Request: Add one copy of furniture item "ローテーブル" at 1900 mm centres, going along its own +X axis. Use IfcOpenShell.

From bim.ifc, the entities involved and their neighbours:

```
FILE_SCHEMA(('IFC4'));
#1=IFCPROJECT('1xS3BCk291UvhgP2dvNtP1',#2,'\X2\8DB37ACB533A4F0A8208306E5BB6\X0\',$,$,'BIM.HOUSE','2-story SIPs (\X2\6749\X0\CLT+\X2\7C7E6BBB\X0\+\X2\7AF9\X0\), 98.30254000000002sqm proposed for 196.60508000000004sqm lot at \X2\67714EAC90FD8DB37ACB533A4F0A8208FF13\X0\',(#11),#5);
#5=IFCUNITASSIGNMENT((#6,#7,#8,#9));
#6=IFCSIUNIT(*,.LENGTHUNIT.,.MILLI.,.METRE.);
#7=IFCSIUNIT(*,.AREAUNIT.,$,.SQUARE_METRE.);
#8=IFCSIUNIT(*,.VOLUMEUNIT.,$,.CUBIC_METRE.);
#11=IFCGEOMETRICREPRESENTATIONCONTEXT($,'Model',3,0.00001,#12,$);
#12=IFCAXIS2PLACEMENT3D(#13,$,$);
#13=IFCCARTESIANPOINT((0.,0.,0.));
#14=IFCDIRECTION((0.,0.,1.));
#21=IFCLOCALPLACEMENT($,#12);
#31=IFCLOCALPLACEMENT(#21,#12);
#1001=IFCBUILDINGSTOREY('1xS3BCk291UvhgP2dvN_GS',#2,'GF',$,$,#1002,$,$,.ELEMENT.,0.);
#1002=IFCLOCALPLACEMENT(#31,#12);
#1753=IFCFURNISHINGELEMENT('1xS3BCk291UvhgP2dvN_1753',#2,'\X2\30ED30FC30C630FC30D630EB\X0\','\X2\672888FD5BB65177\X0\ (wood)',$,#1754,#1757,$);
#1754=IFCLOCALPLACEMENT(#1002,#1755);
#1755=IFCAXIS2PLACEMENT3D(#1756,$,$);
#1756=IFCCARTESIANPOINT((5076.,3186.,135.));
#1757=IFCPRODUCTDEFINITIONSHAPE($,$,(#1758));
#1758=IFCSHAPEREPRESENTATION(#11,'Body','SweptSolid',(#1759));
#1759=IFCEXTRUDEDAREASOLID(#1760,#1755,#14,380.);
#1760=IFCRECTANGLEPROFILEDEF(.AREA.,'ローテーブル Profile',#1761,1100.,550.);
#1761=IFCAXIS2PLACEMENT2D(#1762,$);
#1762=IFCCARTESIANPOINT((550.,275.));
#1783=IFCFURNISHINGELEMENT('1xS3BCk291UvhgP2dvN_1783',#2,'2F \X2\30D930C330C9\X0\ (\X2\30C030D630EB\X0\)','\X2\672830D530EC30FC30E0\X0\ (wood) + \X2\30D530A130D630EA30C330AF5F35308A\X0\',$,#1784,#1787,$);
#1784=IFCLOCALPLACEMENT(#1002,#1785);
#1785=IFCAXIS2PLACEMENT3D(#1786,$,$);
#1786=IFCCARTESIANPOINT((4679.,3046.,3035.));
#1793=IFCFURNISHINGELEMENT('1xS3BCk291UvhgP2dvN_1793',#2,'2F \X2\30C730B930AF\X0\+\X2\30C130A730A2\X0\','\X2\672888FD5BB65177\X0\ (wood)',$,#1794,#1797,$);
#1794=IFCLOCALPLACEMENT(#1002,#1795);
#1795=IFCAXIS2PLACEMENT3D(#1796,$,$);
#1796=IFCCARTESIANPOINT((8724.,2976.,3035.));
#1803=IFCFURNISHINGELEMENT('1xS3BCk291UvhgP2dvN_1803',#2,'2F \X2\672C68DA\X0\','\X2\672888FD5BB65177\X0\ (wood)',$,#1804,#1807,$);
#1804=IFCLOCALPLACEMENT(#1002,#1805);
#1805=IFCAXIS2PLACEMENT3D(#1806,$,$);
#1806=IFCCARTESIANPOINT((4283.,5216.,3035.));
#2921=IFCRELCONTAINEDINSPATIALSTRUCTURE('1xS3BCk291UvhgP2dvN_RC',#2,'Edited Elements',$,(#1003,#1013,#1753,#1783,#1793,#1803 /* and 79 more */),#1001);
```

```python
import ifcopenshell
import ifcopenshell.api.geometry
import ifcopenshell.api.root
import ifcopenshell.util.element
import ifcopenshell.util.placement

model = ifcopenshell.open("bim.ifc")


def reuse_history(source, copy):
    """copy_class also copies each property set's owner history, people and application; keep the originals."""
    for rel in copy.IsDefinedBy:
        if rel.is_a("IfcRelDefinesByProperties") and (history := rel.RelatingPropertyDefinition.OwnerHistory):
            rel.RelatingPropertyDefinition.OwnerHistory = source.OwnerHistory
            ifcopenshell.util.element.remove_deep2(model, history)


source = model.by_guid("1xS3BCk291UvhgP2dvN_1753")
base = ifcopenshell.util.placement.get_local_placement(source.ObjectPlacement)
step = base[:3, 0] * 1900.0

for i in range(1, 2):
    copy = ifcopenshell.api.root.copy_class(model, product=source)
    copy.Representation = ifcopenshell.util.element.copy_deep(
        model, source.Representation, exclude=["IfcGeometricRepresentationContext", "IfcRepresentationMap"]
    )
    reuse_history(source, copy)
    matrix = base.copy()
    matrix[:3, 3] += i * step
    print("added at", matrix[:3, 3].round(3) + 0.0)
    ifcopenshell.api.geometry.edit_object_placement(model, product=copy, matrix=matrix, is_si=False)

model.write("bim_updated.ifc")
```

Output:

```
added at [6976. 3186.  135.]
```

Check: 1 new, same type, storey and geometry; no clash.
